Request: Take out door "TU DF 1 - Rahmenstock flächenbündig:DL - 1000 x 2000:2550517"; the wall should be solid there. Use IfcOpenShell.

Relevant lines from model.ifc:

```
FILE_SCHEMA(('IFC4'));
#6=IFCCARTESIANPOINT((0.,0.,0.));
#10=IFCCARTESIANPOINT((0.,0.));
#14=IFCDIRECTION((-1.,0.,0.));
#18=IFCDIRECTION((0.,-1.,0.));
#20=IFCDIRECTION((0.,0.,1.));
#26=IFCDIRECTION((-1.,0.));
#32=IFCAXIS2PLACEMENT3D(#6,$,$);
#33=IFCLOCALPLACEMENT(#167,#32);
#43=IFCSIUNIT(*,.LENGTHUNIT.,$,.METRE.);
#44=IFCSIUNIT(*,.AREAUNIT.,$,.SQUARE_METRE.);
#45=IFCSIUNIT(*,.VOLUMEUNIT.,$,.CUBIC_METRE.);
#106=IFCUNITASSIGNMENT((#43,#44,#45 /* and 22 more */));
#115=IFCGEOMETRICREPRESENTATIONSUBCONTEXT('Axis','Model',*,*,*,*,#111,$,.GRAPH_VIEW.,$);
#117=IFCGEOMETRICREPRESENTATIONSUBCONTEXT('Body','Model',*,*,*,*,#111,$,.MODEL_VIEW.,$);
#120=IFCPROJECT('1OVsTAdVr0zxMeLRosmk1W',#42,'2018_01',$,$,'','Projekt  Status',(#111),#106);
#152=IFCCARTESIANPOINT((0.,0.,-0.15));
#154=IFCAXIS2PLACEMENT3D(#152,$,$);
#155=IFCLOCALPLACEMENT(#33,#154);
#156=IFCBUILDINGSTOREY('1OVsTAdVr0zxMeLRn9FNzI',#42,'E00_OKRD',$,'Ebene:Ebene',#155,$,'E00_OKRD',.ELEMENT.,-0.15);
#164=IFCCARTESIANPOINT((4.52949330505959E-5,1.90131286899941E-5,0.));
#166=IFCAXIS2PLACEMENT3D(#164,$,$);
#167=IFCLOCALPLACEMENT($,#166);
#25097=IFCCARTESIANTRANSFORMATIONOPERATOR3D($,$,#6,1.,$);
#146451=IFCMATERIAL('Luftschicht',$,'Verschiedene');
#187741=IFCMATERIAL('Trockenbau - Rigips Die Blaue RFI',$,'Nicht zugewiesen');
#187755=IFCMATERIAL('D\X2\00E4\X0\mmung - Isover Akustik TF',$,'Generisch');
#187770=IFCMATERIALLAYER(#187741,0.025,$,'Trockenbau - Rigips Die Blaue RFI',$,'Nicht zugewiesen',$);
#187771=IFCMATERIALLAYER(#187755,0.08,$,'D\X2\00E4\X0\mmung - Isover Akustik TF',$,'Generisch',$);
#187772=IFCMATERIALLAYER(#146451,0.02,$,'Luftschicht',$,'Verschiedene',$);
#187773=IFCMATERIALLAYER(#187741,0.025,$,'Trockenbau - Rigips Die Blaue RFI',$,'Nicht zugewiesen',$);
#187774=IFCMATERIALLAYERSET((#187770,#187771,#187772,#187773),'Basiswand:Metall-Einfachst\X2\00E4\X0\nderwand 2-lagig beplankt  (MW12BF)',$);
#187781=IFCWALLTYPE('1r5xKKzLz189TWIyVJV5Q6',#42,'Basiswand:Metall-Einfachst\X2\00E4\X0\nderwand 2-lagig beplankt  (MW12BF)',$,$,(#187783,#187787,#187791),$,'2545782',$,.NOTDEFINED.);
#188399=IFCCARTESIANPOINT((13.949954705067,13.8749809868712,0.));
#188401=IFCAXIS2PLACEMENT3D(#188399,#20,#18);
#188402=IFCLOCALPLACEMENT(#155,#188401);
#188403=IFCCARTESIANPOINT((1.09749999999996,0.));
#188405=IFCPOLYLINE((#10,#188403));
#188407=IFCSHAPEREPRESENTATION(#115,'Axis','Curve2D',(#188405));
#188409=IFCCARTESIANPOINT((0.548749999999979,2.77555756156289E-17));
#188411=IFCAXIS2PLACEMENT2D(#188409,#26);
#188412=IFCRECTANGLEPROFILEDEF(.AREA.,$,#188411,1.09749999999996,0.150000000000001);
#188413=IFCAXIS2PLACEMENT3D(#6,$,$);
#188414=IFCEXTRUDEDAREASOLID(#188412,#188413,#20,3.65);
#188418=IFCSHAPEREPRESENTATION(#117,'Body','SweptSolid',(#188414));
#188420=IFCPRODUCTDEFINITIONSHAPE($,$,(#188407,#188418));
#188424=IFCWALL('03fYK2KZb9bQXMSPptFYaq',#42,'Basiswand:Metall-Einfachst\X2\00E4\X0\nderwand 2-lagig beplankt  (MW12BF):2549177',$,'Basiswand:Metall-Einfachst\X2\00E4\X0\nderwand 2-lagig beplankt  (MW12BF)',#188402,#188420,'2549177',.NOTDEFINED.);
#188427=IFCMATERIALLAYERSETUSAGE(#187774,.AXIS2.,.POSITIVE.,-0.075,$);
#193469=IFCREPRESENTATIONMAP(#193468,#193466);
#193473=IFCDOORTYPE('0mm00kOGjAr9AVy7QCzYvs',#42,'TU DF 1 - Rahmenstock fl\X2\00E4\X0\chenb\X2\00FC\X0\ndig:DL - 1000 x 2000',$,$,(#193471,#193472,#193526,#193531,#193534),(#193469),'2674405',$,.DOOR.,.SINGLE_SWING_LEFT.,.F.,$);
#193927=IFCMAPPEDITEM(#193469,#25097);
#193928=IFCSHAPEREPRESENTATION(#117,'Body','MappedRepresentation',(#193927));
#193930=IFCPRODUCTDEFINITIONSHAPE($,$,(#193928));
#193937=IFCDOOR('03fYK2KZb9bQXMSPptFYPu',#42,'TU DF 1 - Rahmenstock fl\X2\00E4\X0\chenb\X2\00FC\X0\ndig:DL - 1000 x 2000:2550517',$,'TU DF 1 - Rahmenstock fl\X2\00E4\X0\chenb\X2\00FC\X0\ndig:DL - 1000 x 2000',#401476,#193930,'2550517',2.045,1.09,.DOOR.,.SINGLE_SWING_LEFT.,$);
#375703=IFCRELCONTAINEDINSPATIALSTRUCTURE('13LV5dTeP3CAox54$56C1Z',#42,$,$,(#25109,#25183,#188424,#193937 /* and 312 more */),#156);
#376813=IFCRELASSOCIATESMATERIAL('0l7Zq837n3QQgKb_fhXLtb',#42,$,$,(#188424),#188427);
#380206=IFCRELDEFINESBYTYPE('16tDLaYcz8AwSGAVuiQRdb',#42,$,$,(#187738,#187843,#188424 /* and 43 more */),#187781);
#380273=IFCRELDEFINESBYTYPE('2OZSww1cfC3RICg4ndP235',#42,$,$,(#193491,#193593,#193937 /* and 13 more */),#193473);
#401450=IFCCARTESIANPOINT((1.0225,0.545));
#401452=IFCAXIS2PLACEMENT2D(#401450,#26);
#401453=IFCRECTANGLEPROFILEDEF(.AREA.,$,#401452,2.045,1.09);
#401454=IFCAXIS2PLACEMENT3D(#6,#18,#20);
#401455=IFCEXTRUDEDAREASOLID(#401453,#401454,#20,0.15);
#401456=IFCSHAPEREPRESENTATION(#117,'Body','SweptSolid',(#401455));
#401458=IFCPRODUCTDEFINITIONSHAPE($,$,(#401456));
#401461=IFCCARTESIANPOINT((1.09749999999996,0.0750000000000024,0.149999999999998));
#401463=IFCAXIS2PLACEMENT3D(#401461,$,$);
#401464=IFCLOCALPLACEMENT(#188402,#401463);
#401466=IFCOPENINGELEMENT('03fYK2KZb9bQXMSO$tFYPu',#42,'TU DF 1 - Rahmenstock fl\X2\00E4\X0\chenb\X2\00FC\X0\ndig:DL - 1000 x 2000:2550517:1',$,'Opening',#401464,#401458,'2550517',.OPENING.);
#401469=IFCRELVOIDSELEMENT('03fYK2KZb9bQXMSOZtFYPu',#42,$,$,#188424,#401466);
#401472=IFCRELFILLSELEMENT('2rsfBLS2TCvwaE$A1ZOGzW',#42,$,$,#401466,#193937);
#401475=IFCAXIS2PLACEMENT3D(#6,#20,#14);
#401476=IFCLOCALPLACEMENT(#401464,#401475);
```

```python
import ifcopenshell
import ifcopenshell.api.feature
import ifcopenshell.api.root
import ifcopenshell.geom
import ifcopenshell.util.shape

model = ifcopenshell.open("model.ifc")
settings = ifcopenshell.geom.settings()


def volume(element):
    """Net volume in cubic metres, openings subtracted."""
    shape = ifcopenshell.geom.create_shape(settings, element)
    return ifcopenshell.util.shape.get_volume(shape.geometry)


door = model.by_id(193937)
opening = door.FillsVoids[0].RelatingOpeningElement
wall = opening.VoidsElements[0].RelatingBuildingElement
before = volume(wall)

ifcopenshell.api.root.remove_product(model, product=door)
ifcopenshell.api.feature.remove_feature(model, feature=opening)

after = volume(wall)

print(f"wall volume {before:.3f} -> {after:.3f} m3")

model.write("model_updated.ifc")
```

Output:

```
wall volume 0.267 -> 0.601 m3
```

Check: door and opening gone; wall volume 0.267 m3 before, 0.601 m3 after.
